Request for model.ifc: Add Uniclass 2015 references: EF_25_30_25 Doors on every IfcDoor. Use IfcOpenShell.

First a look at what the model holds.

```python
import ifcopenshell

model = ifcopenshell.open("model.ifc")
print(model.schema)
print("classifications:", [c.Name for c in model.by_type("IfcClassification")])
for ifc_class in ("IfcDoor", "IfcRoof", "IfcStair", "IfcWall", "IfcWindow"):
    print(ifc_class, len(model.by_type(ifc_class)))
```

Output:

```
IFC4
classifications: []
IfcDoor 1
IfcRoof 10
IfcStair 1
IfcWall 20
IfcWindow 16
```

```python
import ifcopenshell
import ifcopenshell.api.classification

model = ifcopenshell.open("model.ifc")

system = ifcopenshell.api.classification.add_classification(model, classification="Uniclass 2015")

codes = {
    "IfcDoor": ("EF_25_30_25", "Doors"),
}
for ifc_class, (code, name) in codes.items():
    products = model.by_type(ifc_class)
    ifcopenshell.api.classification.add_reference(
        model, products=products, classification=system, identification=code, name=name
    )
    print(code, len(products))

model.write("model_rev.ifc")
```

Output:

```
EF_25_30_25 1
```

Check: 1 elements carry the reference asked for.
